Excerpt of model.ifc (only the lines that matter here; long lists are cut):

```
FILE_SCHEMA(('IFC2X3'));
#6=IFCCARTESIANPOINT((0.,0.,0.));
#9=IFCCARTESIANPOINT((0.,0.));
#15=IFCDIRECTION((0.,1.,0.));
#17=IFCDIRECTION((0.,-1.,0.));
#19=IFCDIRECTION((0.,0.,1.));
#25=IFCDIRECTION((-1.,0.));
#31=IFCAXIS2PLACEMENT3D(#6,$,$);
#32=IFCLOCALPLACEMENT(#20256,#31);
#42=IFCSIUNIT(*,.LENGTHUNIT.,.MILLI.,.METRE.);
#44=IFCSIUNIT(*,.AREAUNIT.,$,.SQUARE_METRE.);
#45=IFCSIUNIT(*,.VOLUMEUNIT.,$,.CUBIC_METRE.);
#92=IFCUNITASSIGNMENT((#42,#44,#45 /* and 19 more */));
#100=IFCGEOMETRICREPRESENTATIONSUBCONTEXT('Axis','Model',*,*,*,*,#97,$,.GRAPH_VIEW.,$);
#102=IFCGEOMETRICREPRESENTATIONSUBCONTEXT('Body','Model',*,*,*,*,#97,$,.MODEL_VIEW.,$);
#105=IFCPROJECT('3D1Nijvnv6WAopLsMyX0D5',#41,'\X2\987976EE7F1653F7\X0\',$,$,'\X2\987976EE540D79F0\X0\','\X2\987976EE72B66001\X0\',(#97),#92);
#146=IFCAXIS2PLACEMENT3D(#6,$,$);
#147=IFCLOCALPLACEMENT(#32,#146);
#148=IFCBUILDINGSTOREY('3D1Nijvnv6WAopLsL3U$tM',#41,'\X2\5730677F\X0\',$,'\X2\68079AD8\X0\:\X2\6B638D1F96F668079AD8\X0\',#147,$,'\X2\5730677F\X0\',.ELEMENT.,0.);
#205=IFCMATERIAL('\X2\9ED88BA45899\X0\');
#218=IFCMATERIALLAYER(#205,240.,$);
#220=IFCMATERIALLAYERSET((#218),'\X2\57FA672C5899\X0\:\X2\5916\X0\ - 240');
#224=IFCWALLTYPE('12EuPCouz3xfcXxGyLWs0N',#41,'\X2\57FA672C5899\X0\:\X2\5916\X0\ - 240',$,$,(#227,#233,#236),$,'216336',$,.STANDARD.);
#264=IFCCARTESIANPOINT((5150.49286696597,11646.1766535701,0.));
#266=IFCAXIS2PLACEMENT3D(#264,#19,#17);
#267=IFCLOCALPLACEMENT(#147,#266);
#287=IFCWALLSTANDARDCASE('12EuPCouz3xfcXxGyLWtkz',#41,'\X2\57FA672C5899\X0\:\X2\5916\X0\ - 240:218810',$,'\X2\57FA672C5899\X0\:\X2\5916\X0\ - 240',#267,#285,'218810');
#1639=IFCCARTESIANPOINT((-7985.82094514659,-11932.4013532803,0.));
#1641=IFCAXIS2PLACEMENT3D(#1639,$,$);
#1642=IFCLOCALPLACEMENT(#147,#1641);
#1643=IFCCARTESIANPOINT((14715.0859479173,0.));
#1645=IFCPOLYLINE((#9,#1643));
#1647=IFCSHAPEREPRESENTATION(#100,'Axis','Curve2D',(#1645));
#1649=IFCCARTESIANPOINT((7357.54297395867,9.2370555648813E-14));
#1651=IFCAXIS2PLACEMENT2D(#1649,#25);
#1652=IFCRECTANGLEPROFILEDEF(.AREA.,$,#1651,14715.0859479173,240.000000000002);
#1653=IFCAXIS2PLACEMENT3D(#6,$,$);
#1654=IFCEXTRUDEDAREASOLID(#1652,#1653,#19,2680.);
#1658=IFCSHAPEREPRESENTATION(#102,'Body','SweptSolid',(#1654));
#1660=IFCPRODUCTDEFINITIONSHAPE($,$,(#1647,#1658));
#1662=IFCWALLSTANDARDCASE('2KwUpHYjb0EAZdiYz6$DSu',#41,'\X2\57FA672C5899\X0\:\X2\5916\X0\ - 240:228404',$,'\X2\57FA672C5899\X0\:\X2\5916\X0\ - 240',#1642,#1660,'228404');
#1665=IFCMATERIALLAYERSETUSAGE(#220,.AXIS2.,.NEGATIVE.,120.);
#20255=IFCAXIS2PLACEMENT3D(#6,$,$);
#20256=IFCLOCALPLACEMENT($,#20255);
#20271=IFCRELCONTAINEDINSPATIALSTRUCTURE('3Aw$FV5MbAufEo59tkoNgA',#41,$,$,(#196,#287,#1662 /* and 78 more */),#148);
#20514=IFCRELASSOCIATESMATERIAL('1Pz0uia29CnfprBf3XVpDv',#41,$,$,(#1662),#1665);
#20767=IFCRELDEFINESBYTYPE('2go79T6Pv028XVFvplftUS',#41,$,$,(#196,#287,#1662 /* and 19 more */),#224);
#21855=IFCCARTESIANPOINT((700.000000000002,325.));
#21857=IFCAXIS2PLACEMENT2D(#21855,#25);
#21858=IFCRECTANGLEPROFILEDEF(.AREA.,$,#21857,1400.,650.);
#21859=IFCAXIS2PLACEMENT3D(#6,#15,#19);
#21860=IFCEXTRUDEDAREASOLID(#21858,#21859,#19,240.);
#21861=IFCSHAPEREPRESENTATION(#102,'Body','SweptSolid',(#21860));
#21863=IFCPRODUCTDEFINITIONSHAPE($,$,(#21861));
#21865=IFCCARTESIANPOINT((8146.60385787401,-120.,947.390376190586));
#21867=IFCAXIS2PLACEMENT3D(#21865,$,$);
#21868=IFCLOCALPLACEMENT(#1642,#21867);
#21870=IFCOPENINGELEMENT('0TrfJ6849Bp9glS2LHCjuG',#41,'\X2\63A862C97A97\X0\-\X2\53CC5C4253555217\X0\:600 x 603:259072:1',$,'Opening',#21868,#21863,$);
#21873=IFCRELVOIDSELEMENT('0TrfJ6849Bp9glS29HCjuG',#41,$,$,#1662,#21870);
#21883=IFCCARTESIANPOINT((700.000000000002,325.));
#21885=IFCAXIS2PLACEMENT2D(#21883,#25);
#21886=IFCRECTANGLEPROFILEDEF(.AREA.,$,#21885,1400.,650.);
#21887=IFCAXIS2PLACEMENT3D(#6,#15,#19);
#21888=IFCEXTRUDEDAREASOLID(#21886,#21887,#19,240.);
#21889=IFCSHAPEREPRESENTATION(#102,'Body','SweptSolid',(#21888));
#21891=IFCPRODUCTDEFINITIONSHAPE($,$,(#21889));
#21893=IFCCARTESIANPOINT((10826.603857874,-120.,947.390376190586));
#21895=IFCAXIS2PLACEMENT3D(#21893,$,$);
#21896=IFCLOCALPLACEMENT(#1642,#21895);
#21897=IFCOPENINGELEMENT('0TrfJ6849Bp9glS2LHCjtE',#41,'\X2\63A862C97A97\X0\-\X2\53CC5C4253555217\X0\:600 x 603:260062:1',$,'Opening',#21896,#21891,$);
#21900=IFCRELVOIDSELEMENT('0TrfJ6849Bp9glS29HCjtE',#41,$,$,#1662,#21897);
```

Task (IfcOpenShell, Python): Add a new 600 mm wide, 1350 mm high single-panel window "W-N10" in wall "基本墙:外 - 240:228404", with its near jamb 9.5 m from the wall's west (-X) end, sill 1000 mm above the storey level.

```python
import numpy as np
import ifcopenshell
import ifcopenshell.api.feature
import ifcopenshell.api.geometry
import ifcopenshell.api.root
import ifcopenshell.api.spatial
import ifcopenshell.api.type
import ifcopenshell.geom
import ifcopenshell.util.element
import ifcopenshell.util.placement
import ifcopenshell.util.representation
import ifcopenshell.util.shape
import ifcopenshell.util.unit

model = ifcopenshell.open("model.ifc")
unit_scale = ifcopenshell.util.unit.calculate_unit_scale(model)
settings = ifcopenshell.geom.settings()


def volume(element):
    """Net volume in cubic metres, openings subtracted."""
    shape = ifcopenshell.geom.create_shape(settings, element)
    return ifcopenshell.util.shape.get_volume(shape.geometry)


wall = model.by_id(1662)
storey = ifcopenshell.util.element.get_container(wall, ifc_class="IfcBuildingStorey")
context = ifcopenshell.util.representation.get_context(model, "Model", "Body", "MODEL_VIEW")
before = volume(wall)

width, height, from_end, sill = 0.6, 1.35, 9.5, 1  # metres

# The wall runs along its own X axis, and the end named is its -X end.
wall_shape = ifcopenshell.geom.create_shape(settings, wall)
x, y, z = ifcopenshell.util.shape.get_vertices(wall_shape.geometry).T
start = x.min() + from_end
face, thickness = float(y.min()), float(y.max() - y.min())
wall_matrix = ifcopenshell.util.placement.get_local_placement(wall.ObjectPlacement)
level = ifcopenshell.util.placement.get_local_placement(storey.ObjectPlacement)[2, 3]


def in_wall(x, y):
    """Placement at x, y metres in the wall's axes, at sill height."""
    matrix = wall_matrix.copy()
    matrix[:, 3] = wall_matrix @ np.array([x / unit_scale, y / unit_scale, 0.0, 1.0])
    matrix[2, 3] = level + sill / unit_scale
    return matrix


# Opening: a box that overshoots both wall faces by 50 mm.
opening = ifcopenshell.api.root.create_entity(model, ifc_class="IfcOpeningElement")
box = ifcopenshell.api.geometry.add_wall_representation(
    model, context=context, length=width, height=height, thickness=thickness + 0.1
)
ifcopenshell.api.geometry.assign_representation(model, product=opening, representation=box)
ifcopenshell.api.geometry.edit_object_placement(model, product=opening, matrix=in_wall(start, face - 0.05), is_si=False)
ifcopenshell.api.feature.add_feature(model, feature=opening, element=wall)

window = ifcopenshell.api.root.create_entity(model, ifc_class="IfcWindow", name="W-N10")
window.OverallWidth, window.OverallHeight = width / unit_scale, height / unit_scale
body = ifcopenshell.api.geometry.add_window_representation(
    model,
    context=context,
    overall_width=window.OverallWidth,
    overall_height=window.OverallHeight,
    partition_type="SINGLE_PANEL",
)
ifcopenshell.api.geometry.assign_representation(model, product=window, representation=body)
ifcopenshell.api.spatial.assign_container(model, products=[window], relating_structure=storey)
fills = ifcopenshell.api.feature.add_filling(model, opening=opening, element=window)
fills.OwnerHistory = window.OwnerHistory  # required in IFC2X3

# IFC2X3 keeps the operation on the window style.
style = ifcopenshell.api.root.create_entity(model, ifc_class="IfcWindowStyle", name="W-N10")
style.OperationType, style.ConstructionType = "SINGLE_PANEL", "NOTDEFINED"
style.ParameterTakesPrecedence = style.Sizeable = False
ifcopenshell.api.type.assign_type(model, related_objects=[window], relating_type=style)

# Centre the window in the wall's thickness.
ifcopenshell.api.geometry.edit_object_placement(model, product=window, matrix=in_wall(start, face), is_si=False)
window_shape = ifcopenshell.geom.create_shape(settings, window)
depth = ifcopenshell.util.shape.get_vertices(window_shape.geometry)[:, 1]
offset = face + thickness / 2 - (depth.min() + depth.max()) / 2
ifcopenshell.api.geometry.edit_object_placement(model, product=window, matrix=in_wall(start, offset), is_si=False)

after = volume(wall)

print(f"wall volume {before:.3f} -> {after:.3f} m3")

model.write("model-out.ifc")
```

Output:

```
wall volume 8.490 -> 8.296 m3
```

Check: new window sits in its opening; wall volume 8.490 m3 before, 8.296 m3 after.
